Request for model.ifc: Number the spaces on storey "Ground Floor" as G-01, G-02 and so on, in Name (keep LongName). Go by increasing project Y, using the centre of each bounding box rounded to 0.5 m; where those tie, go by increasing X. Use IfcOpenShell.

First a look at what the model holds.

```python
import ifcopenshell
import ifcopenshell.util.element
import ifcopenshell.util.placement

model = ifcopenshell.open("model.ifc")
print(model.schema)
storey = next(s for s in model.by_type("IfcBuildingStorey") if s.Name == "Ground Floor")
spaces = [e for e in ifcopenshell.util.element.get_decomposition(storey) if e.is_a("IfcSpace")]
for e in sorted(spaces, key=lambda e: e.id()):
    origin = ifcopenshell.util.placement.get_local_placement(e.ObjectPlacement)[:3, 3]
    print(e.id(), e.Name, e.LongName, origin.round(2) + 0.0, sep=" | ")
```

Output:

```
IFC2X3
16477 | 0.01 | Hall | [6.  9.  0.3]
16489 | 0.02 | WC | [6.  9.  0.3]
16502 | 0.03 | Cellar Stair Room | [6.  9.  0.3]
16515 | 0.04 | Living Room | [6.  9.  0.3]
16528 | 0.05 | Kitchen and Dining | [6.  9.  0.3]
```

```python
import ifcopenshell
import ifcopenshell.geom
import ifcopenshell.util.element
import ifcopenshell.util.shape

model = ifcopenshell.open("model.ifc")
settings = ifcopenshell.geom.settings()
settings.set("use-world-coords", True)


def centre(element):
    shape = ifcopenshell.geom.create_shape(settings, element)
    return ifcopenshell.util.shape.get_bbox_centroid(shape.geometry)


storey = next(s for s in model.by_type("IfcBuildingStorey") if s.Name == "Ground Floor")
spaces = [e for e in ifcopenshell.util.element.get_decomposition(storey) if e.is_a("IfcSpace")]

# Insertion points can sit at a corner or the storey origin, so sort by the geometry (in metres).
centres = {e: centre(e) for e in spaces}
spaces.sort(key=lambda e: (round(centres[e][1] / 0.5), centres[e][0]))

for i, e in enumerate(spaces, start=1):
    number = f"G-{i:02d}"
    e.Name = number
    print(e.id(), number)

model.write("model_rev.ifc")
```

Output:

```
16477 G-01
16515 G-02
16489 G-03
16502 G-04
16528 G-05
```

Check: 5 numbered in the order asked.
